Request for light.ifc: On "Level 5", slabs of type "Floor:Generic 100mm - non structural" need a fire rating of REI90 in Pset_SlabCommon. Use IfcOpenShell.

First a look at what the model holds.

```python
import ifcopenshell
import ifcopenshell.util.element

model = ifcopenshell.open("light.ifc")
print(model.schema)
storey = next(s for s in model.by_type("IfcBuildingStorey") if s.Name == "Level 5")
slabs = [e for e in ifcopenshell.util.element.get_decomposition(storey) if e.is_a("IfcSlab")]
seen = {}
for e in slabs:
    element_type = ifcopenshell.util.element.get_type(e)
    key = (element_type.Name if element_type != e and element_type else None, ifcopenshell.util.element.get_pset(e, "Pset_SlabCommon", "FireRating"))
    seen[key] = seen.get(key, 0) + 1
for (name, value), count in sorted(seen.items(), key=str):
    print(count, "x", name, "|", value)
```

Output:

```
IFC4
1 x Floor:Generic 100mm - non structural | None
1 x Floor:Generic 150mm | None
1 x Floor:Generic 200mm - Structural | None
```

```python
import ifcopenshell
import ifcopenshell.api.pset
import ifcopenshell.util.element

model = ifcopenshell.open("light.ifc")

storey = next(s for s in model.by_type("IfcBuildingStorey") if s.Name == "Level 5")
slabs = [e for e in ifcopenshell.util.element.get_decomposition(storey) if e.is_a("IfcSlab")]

count = 0
for e in slabs:
    element_type = ifcopenshell.util.element.get_type(e)
    if element_type in (None, e) or element_type.Name != "Floor:Generic 100mm - non structural":
        continue
    # add_pset returns the element's existing set when there is one.
    pset = ifcopenshell.api.pset.add_pset(model, product=e, name="Pset_SlabCommon")
    ifcopenshell.api.pset.edit_pset(model, pset=pset, properties={"FireRating": "REI90"})
    count += 1

print(count, "slabs updated")

model.write("light-out.ifc")
```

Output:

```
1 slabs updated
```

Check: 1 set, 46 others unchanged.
